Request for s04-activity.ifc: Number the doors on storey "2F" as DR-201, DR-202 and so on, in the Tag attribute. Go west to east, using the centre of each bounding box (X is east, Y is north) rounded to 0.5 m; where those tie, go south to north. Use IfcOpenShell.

First a look at what the model holds.

```python
import ifcopenshell
import ifcopenshell.util.element
import ifcopenshell.util.placement

model = ifcopenshell.open("s04-activity.ifc")
print(model.schema)
storey = next(s for s in model.by_type("IfcBuildingStorey") if s.Name == "2F")
doors = [e for e in ifcopenshell.util.element.get_decomposition(storey) if e.is_a("IfcDoor")]
for e in sorted(doors, key=lambda e: e.id()):
    origin = ifcopenshell.util.placement.get_local_placement(e.ObjectPlacement)[:3, 3]
    print(e.id(), e.Tag, e.Name, origin.round(2) + 0.0, sep=" | ")
```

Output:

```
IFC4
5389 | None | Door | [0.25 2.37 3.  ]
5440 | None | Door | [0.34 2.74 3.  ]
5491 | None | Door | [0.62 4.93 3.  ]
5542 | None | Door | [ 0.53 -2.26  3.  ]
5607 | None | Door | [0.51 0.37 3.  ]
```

```python
import ifcopenshell
import ifcopenshell.geom
import ifcopenshell.util.element
import ifcopenshell.util.shape

model = ifcopenshell.open("s04-activity.ifc")
settings = ifcopenshell.geom.settings()
settings.set("use-world-coords", True)


def centre(element):
    shape = ifcopenshell.geom.create_shape(settings, element)
    return ifcopenshell.util.shape.get_bbox_centroid(shape.geometry)


storey = next(s for s in model.by_type("IfcBuildingStorey") if s.Name == "2F")
doors = [e for e in ifcopenshell.util.element.get_decomposition(storey) if e.is_a("IfcDoor")]

# Insertion points can sit at a corner or the storey origin, so sort by the geometry (in metres).
centres = {e: centre(e) for e in doors}
doors.sort(key=lambda e: (round(centres[e][0] / 0.5), centres[e][1]))

for i, e in enumerate(doors, start=1):
    number = f"DR-2{i:02d}"
    e.Tag = number
    print(e.id(), number)

model.write("s04-activity_edited.ifc")
```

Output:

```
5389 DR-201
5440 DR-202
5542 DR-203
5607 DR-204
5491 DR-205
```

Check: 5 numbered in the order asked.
